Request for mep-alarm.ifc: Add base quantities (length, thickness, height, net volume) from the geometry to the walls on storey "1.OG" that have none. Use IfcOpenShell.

First a look at what the model holds.

```python
import ifcopenshell
import ifcopenshell.util.element
import ifcopenshell.util.unit

model = ifcopenshell.open("mep-alarm.ifc")
print(model.schema)
for unit_type in ("LENGTHUNIT", "AREAUNIT", "VOLUMEUNIT"):
    print(unit_type, ifcopenshell.util.unit.calculate_unit_scale(model, unit_type))
storey = next(s for s in model.by_type("IfcBuildingStorey") if s.Name == "1.OG")
walls = [e for e in ifcopenshell.util.element.get_decomposition(storey) if e.is_a("IfcWall")]
for e in sorted(walls, key=lambda e: e.id()):
    print(e.id(), e.is_a(), e.Name, list(ifcopenshell.util.element.get_psets(e, qtos_only=True)), sep=" | ")
```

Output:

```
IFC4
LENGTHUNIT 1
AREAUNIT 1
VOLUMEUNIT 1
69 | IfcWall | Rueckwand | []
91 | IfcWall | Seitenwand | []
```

```python
import ifcopenshell
import ifcopenshell.api.pset
import ifcopenshell.geom
import ifcopenshell.util.element
import ifcopenshell.util.shape
import ifcopenshell.util.unit

model = ifcopenshell.open("mep-alarm.ifc")
unit_scale = ifcopenshell.util.unit.calculate_unit_scale(model)
volume_scale = ifcopenshell.util.unit.calculate_unit_scale(model, "VOLUMEUNIT")
settings = ifcopenshell.geom.settings()

storey = next(s for s in model.by_type("IfcBuildingStorey") if s.Name == "1.OG")
walls = [e for e in ifcopenshell.util.element.get_decomposition(storey) if e.is_a("IfcWall")]

for e in sorted(walls, key=lambda e: e.id()):
    if ifcopenshell.util.element.get_psets(e, qtos_only=True, should_inherit=False):
        continue
    # Geometry comes back in metres, in the element's own axes.
    shape = ifcopenshell.geom.create_shape(settings, e)
    values = {
        "Length": ifcopenshell.util.shape.get_x(shape.geometry) / unit_scale,
        "Width": ifcopenshell.util.shape.get_y(shape.geometry) / unit_scale,
        "Height": ifcopenshell.util.shape.get_z(shape.geometry) / unit_scale,
        "NetVolume": ifcopenshell.util.shape.get_volume(shape.geometry) / volume_scale,
    }
    qto = ifcopenshell.api.pset.add_qto(model, product=e, name="Qto_WallBaseQuantities")
    ifcopenshell.api.pset.edit_qto(model, qto=qto, properties=values)
    print(e.id(), {k: round(v, 3) for k, v in values.items()})

model.write("mep-alarm-out.ifc")
```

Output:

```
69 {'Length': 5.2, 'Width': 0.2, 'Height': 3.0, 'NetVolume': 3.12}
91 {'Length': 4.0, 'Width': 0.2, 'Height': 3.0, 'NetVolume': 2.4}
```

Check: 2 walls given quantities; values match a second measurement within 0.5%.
